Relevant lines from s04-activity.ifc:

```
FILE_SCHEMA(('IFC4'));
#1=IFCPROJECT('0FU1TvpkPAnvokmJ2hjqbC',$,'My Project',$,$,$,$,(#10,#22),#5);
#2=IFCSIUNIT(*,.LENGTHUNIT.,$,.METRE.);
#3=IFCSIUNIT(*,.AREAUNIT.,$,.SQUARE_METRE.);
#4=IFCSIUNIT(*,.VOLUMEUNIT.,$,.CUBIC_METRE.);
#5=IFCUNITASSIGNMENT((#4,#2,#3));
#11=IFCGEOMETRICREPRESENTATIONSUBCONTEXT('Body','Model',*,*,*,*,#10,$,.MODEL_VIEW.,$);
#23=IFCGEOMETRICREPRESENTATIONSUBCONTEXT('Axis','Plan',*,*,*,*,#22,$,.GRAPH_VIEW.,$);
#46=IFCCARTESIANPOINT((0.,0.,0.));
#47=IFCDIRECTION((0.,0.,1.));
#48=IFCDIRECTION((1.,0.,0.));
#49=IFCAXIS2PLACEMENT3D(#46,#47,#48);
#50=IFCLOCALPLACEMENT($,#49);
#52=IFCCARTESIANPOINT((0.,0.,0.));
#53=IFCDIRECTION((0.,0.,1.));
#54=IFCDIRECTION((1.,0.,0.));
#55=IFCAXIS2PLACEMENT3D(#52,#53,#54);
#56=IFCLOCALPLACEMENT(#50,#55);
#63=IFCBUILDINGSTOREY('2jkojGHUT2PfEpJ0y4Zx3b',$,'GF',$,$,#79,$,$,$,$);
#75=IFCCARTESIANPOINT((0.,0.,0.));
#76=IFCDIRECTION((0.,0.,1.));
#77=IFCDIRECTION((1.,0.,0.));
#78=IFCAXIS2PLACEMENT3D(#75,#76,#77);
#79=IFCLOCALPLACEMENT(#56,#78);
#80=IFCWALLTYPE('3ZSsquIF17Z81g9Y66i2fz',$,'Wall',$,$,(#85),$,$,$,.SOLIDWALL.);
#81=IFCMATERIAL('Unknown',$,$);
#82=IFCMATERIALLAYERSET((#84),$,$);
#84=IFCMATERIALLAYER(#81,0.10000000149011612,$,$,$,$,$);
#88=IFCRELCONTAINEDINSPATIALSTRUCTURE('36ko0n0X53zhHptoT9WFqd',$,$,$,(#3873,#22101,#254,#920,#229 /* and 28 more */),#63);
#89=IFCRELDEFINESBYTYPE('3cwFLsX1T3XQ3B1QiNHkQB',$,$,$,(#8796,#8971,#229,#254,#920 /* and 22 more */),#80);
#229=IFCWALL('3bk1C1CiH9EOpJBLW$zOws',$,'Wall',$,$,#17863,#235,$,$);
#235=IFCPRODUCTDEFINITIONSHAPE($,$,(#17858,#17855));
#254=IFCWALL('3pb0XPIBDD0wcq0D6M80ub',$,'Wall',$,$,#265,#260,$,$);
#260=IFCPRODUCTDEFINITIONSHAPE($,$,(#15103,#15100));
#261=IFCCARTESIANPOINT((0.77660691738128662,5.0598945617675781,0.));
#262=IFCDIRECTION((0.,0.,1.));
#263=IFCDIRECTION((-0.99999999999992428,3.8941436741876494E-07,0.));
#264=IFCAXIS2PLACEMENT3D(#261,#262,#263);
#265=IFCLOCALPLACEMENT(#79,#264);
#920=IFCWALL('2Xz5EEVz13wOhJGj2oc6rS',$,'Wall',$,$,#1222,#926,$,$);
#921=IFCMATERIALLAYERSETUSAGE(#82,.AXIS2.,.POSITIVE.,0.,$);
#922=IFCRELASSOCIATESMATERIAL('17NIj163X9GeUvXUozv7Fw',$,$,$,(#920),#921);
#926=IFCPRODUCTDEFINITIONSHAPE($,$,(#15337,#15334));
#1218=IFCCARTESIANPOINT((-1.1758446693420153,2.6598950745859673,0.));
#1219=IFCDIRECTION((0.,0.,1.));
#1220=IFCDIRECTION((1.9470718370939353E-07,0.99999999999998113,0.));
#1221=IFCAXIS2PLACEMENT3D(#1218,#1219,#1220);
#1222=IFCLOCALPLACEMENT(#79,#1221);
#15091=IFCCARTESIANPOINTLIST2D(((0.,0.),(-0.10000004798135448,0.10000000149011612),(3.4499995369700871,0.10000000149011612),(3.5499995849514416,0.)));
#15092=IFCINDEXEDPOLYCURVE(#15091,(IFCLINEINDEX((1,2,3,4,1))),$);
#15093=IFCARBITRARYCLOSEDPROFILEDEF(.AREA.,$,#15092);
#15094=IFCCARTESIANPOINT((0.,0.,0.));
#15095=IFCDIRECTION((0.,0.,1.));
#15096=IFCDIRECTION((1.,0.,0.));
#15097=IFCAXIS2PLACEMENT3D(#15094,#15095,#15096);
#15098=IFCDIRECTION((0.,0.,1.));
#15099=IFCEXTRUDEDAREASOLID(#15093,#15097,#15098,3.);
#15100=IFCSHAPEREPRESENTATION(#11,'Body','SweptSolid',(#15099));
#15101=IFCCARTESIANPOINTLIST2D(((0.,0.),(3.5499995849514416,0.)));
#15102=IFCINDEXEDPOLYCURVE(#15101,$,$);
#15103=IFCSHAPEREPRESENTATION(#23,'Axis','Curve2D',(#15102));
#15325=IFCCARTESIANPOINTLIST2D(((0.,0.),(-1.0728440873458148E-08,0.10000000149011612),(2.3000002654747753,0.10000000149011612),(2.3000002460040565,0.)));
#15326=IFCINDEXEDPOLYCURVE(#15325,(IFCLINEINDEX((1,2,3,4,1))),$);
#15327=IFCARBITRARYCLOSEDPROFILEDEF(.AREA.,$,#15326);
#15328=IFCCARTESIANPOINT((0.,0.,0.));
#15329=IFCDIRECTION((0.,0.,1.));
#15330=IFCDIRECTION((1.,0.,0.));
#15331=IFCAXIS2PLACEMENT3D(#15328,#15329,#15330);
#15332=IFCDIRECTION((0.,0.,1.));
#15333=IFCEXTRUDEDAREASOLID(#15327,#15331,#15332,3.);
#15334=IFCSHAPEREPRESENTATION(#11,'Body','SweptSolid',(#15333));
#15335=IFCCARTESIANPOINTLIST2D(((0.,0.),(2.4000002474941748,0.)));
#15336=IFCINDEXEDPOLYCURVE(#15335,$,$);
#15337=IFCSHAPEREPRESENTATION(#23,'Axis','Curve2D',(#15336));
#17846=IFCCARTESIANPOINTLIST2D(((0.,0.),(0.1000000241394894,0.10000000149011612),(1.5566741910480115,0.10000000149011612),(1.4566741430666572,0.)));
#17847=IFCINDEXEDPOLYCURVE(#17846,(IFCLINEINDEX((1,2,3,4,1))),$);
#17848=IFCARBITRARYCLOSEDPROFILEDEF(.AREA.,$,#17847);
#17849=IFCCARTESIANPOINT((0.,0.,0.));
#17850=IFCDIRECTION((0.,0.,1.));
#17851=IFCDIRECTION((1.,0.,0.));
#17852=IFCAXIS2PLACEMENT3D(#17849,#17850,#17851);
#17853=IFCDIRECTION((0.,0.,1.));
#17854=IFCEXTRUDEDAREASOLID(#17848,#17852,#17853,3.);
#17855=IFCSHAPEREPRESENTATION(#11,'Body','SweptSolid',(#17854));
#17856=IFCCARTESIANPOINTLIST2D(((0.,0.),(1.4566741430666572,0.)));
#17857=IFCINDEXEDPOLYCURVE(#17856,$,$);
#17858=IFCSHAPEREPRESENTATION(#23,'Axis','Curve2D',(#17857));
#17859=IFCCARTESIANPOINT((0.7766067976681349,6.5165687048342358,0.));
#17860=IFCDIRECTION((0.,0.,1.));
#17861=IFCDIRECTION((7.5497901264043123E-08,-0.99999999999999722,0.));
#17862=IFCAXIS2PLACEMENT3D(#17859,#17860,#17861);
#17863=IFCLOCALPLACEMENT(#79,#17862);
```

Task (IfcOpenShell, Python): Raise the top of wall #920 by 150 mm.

```python
import ifcopenshell
import ifcopenshell.geom
import ifcopenshell.util.representation
import ifcopenshell.util.shape
import ifcopenshell.util.unit

model = ifcopenshell.open("s04-activity.ifc")
unit_scale = ifcopenshell.util.unit.calculate_unit_scale(model)
settings = ifcopenshell.geom.settings()


def volume(element):
    """Net volume in cubic metres, openings subtracted."""
    shape = ifcopenshell.geom.create_shape(settings, element)
    return ifcopenshell.util.shape.get_volume(shape.geometry)


wall = model.by_guid("2Xz5EEVz13wOhJGj2oc6rS")
before = volume(wall)

body = ifcopenshell.util.representation.get_representation(wall, "Model", "Body")
solid = body.Items[0]
old_height = solid.Depth
solid.Depth += 0.15 / unit_scale
after = volume(wall)

print(f"height {old_height:g} -> {solid.Depth:g}, volume {before:.3f} -> {after:.3f} m3")

model.write("s04-activity-out.ifc")
```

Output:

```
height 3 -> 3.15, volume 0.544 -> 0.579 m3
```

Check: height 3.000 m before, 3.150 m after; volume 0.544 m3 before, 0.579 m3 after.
